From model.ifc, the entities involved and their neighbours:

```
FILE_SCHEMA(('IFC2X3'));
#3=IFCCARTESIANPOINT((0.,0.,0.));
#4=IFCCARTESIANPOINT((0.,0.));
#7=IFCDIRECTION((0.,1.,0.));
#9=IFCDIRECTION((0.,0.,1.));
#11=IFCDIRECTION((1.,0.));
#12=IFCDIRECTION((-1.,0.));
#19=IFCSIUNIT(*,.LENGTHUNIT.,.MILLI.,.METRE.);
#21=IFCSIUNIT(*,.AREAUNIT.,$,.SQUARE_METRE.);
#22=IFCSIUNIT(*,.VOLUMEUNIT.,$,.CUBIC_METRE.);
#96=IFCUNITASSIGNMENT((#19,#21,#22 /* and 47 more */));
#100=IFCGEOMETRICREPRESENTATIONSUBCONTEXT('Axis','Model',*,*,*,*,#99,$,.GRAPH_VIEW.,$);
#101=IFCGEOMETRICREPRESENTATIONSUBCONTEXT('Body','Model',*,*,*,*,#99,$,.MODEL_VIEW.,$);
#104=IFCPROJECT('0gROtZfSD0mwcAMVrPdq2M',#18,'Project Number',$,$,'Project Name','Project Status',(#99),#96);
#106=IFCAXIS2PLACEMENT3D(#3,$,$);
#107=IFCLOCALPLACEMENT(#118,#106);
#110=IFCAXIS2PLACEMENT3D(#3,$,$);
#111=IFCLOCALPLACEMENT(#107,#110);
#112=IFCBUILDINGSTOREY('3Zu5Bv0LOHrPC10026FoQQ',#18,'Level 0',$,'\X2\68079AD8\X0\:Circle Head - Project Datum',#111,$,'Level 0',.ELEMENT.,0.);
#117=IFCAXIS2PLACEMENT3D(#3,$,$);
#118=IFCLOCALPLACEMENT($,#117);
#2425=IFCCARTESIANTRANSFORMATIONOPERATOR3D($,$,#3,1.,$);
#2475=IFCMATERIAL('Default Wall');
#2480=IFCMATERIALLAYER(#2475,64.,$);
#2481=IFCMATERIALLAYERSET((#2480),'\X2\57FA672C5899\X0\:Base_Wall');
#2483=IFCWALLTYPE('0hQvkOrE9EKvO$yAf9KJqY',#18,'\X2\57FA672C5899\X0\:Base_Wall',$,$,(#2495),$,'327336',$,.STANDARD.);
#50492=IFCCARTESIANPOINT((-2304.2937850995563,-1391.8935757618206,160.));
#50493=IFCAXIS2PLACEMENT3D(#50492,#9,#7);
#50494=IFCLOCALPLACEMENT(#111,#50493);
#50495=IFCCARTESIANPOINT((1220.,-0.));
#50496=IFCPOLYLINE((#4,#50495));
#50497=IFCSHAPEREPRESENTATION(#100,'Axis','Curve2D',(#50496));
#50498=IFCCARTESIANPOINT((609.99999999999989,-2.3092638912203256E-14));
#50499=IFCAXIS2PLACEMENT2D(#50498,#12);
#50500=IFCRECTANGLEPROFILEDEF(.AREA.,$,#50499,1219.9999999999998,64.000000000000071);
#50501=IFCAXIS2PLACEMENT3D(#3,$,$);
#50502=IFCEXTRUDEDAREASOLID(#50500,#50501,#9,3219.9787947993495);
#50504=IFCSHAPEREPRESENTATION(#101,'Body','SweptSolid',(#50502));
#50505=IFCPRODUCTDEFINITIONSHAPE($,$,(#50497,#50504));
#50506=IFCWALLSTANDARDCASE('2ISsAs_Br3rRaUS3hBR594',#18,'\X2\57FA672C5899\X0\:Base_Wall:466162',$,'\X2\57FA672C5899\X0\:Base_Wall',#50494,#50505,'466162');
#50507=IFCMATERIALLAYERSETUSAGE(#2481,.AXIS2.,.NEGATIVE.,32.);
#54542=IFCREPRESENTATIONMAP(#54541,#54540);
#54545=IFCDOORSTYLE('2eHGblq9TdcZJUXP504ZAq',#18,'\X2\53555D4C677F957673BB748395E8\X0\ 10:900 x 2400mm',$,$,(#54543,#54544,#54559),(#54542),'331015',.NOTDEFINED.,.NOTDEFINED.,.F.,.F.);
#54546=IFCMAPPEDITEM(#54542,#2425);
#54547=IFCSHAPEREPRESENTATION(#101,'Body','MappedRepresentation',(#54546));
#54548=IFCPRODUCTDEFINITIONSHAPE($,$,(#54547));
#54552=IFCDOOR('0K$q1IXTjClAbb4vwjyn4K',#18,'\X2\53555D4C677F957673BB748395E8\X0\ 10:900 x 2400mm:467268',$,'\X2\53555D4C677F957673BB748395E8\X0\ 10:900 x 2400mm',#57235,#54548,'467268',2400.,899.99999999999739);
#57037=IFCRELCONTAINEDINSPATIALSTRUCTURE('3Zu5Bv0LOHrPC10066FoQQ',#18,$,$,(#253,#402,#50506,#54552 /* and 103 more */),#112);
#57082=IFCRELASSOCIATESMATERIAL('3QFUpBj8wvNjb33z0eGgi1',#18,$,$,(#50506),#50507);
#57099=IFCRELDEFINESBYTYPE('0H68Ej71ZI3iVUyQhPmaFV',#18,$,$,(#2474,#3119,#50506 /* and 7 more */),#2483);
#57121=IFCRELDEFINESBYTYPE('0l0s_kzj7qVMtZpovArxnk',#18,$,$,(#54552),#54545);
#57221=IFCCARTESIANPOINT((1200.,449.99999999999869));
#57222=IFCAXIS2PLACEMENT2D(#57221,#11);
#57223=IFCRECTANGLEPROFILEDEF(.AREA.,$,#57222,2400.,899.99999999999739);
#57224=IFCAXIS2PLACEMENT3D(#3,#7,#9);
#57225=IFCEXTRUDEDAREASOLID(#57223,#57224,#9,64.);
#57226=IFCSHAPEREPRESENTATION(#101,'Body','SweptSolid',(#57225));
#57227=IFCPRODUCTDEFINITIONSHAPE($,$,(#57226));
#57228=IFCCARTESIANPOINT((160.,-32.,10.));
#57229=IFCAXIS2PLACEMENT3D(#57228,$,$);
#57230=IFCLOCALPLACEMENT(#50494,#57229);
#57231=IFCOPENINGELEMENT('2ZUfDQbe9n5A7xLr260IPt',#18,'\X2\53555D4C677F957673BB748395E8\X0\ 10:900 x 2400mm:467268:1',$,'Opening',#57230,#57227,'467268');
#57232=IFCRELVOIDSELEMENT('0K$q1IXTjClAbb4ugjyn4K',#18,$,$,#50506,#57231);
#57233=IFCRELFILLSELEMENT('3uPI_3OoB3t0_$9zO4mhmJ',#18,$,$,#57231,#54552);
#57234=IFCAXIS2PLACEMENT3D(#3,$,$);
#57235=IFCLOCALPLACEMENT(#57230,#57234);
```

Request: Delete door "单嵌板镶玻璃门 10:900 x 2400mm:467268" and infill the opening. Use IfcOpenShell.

```python
import ifcopenshell
import ifcopenshell.api.feature
import ifcopenshell.api.root
import ifcopenshell.geom
import ifcopenshell.util.shape

model = ifcopenshell.open("model.ifc")
settings = ifcopenshell.geom.settings()


def volume(element):
    """Net volume in cubic metres, openings subtracted."""
    shape = ifcopenshell.geom.create_shape(settings, element)
    return ifcopenshell.util.shape.get_volume(shape.geometry)


door = model.by_guid("0K$q1IXTjClAbb4vwjyn4K")
opening = door.FillsVoids[0].RelatingOpeningElement
wall = opening.VoidsElements[0].RelatingBuildingElement
before = volume(wall)

ifcopenshell.api.root.remove_product(model, product=door)
ifcopenshell.api.feature.remove_feature(model, feature=opening)

after = volume(wall)

print(f"wall volume {before:.3f} -> {after:.3f} m3")

model.write("model_v2.ifc")
```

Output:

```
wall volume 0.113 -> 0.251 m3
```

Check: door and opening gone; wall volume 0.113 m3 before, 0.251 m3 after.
